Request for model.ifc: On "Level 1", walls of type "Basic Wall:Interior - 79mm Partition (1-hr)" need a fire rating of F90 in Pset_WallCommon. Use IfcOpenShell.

First a look at what the model holds.

```python
import ifcopenshell
import ifcopenshell.util.element

model = ifcopenshell.open("model.ifc")
print(model.schema)
storey = next(s for s in model.by_type("IfcBuildingStorey") if s.Name == "Level 1")
walls = [e for e in ifcopenshell.util.element.get_decomposition(storey) if e.is_a("IfcWall")]
seen = {}
for e in walls:
    element_type = ifcopenshell.util.element.get_type(e)
    key = (element_type.Name if element_type != e and element_type else None, ifcopenshell.util.element.get_pset(e, "Pset_WallCommon", "FireRating"))
    seen[key] = seen.get(key, 0) + 1
for (name, value), count in sorted(seen.items(), key=str):
    print(count, "x", name, "|", value)
```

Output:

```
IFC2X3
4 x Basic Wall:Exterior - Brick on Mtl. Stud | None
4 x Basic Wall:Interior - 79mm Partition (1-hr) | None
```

```python
import ifcopenshell
import ifcopenshell.api.pset
import ifcopenshell.util.element

model = ifcopenshell.open("model.ifc")

storey = next(s for s in model.by_type("IfcBuildingStorey") if s.Name == "Level 1")
walls = [e for e in ifcopenshell.util.element.get_decomposition(storey) if e.is_a("IfcWall")]

count = 0
for e in walls:
    element_type = ifcopenshell.util.element.get_type(e)
    if element_type in (None, e) or element_type.Name != "Basic Wall:Interior - 79mm Partition (1-hr)":
        continue
    # add_pset returns the element's existing set when there is one.
    pset = ifcopenshell.api.pset.add_pset(model, product=e, name="Pset_WallCommon")
    ifcopenshell.api.pset.edit_pset(model, pset=pset, properties={"FireRating": "F90"})
    count += 1

print(count, "walls updated")

model.write("model_updated.ifc")
```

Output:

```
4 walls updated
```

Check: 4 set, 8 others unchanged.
